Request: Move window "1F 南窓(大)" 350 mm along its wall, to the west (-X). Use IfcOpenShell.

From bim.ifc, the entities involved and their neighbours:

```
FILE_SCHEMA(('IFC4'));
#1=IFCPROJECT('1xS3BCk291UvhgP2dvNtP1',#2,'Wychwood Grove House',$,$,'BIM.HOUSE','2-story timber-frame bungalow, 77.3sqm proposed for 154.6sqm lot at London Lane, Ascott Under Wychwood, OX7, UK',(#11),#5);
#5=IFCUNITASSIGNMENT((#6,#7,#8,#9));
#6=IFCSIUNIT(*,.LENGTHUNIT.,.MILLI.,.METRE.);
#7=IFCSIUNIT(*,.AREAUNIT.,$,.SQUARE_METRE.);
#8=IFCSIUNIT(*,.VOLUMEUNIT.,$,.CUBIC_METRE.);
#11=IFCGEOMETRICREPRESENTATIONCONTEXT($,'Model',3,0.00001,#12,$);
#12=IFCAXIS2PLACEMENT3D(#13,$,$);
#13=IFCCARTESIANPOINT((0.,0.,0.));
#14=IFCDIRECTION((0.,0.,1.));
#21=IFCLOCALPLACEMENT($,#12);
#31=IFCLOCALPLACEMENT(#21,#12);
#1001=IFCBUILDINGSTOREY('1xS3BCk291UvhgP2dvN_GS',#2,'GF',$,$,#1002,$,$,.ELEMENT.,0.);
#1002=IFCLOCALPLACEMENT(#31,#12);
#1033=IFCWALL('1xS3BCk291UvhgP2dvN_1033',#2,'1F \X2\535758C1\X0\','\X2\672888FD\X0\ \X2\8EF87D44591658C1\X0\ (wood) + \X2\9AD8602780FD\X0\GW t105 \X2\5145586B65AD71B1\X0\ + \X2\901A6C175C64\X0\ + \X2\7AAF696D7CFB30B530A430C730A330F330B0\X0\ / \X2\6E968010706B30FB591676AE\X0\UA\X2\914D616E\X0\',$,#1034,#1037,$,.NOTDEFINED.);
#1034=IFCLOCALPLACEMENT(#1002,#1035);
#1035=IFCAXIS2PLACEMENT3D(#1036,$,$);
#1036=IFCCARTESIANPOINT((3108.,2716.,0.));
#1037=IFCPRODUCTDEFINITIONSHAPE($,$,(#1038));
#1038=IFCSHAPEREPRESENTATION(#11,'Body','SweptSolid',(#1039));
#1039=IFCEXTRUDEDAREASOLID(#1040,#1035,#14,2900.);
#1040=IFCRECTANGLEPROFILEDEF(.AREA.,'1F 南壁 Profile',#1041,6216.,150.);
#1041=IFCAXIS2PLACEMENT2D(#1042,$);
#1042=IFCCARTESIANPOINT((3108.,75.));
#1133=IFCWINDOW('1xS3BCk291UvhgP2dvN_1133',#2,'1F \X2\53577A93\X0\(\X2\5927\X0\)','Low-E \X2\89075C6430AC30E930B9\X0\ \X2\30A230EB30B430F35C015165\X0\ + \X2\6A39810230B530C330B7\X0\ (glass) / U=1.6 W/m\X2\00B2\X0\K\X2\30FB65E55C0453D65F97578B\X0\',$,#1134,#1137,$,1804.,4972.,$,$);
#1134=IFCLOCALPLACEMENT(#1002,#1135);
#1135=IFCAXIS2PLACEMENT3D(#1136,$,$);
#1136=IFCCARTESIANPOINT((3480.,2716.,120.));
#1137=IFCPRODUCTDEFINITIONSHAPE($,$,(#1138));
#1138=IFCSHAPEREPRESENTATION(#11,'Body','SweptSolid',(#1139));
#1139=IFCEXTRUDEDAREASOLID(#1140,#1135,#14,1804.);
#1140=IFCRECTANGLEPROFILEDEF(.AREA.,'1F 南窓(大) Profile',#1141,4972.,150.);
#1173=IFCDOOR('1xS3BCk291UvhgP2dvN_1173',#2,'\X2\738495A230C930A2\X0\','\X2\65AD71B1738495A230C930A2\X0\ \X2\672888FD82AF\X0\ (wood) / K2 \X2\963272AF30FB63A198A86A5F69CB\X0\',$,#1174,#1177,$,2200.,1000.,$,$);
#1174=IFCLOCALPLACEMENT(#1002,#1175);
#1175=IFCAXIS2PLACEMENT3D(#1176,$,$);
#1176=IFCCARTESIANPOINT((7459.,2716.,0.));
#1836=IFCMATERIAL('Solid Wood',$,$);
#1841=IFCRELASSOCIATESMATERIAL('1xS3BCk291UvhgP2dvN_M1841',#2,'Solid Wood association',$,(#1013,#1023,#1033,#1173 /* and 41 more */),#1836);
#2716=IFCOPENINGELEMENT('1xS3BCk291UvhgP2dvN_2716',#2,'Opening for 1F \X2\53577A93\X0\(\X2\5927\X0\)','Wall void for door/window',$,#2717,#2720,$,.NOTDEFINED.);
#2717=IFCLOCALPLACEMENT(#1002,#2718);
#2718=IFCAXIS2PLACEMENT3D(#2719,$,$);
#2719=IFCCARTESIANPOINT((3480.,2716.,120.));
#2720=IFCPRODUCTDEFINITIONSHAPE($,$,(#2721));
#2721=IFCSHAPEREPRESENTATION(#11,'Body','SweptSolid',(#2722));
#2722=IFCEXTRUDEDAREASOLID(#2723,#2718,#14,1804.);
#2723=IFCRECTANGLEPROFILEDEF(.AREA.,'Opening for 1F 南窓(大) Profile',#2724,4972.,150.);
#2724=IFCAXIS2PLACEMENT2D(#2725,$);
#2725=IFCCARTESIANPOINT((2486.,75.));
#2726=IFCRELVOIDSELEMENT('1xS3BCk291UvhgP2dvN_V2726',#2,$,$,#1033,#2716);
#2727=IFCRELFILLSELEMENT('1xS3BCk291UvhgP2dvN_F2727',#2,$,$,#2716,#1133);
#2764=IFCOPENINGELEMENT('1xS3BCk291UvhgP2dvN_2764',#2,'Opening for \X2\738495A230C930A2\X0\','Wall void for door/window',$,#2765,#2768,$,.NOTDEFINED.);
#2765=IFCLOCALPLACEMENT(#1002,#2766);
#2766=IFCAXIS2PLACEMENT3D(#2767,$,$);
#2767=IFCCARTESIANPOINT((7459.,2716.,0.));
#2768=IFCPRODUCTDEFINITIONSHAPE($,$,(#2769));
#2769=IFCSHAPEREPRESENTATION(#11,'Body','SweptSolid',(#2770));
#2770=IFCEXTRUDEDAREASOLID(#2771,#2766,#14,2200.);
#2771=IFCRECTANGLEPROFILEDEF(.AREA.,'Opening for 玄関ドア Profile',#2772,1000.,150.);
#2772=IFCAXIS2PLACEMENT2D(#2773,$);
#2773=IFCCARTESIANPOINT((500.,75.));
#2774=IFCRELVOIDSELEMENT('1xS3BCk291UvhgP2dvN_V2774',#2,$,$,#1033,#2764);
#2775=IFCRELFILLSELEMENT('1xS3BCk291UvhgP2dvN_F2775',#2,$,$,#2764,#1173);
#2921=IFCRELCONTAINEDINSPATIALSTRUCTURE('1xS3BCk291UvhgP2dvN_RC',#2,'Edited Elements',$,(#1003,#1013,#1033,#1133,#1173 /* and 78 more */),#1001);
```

```python
import ifcopenshell
import ifcopenshell.api.geometry
import ifcopenshell.util.placement
import ifcopenshell.util.unit

model = ifcopenshell.open("bim.ifc")
unit_scale = ifcopenshell.util.unit.calculate_unit_scale(model)

window = model.by_guid("1xS3BCk291UvhgP2dvN_1133")
opening = window.FillsVoids[0].RelatingOpeningElement
wall = opening.VoidsElements[0].RelatingBuildingElement

wall_matrix = ifcopenshell.util.placement.get_local_placement(wall.ObjectPlacement)
shift = wall_matrix[:3, 0] * -0.35 / unit_scale
before = ifcopenshell.util.placement.get_local_placement(window.ObjectPlacement)[:3, 3].copy()

# The window is not placed relative to its opening, so move both.
for product in (opening, window):
    matrix = ifcopenshell.util.placement.get_local_placement(product.ObjectPlacement)
    matrix[:3, 3] += shift
    ifcopenshell.api.geometry.edit_object_placement(model, product=product, matrix=matrix, is_si=False)

after = ifcopenshell.util.placement.get_local_placement(window.ObjectPlacement)[:3, 3]
print("window moved by", (after - before).round(3) + 0.0)

model.write("bim_edited.ifc")
```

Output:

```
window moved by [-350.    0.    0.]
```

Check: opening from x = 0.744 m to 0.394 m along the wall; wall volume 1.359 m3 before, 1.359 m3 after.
